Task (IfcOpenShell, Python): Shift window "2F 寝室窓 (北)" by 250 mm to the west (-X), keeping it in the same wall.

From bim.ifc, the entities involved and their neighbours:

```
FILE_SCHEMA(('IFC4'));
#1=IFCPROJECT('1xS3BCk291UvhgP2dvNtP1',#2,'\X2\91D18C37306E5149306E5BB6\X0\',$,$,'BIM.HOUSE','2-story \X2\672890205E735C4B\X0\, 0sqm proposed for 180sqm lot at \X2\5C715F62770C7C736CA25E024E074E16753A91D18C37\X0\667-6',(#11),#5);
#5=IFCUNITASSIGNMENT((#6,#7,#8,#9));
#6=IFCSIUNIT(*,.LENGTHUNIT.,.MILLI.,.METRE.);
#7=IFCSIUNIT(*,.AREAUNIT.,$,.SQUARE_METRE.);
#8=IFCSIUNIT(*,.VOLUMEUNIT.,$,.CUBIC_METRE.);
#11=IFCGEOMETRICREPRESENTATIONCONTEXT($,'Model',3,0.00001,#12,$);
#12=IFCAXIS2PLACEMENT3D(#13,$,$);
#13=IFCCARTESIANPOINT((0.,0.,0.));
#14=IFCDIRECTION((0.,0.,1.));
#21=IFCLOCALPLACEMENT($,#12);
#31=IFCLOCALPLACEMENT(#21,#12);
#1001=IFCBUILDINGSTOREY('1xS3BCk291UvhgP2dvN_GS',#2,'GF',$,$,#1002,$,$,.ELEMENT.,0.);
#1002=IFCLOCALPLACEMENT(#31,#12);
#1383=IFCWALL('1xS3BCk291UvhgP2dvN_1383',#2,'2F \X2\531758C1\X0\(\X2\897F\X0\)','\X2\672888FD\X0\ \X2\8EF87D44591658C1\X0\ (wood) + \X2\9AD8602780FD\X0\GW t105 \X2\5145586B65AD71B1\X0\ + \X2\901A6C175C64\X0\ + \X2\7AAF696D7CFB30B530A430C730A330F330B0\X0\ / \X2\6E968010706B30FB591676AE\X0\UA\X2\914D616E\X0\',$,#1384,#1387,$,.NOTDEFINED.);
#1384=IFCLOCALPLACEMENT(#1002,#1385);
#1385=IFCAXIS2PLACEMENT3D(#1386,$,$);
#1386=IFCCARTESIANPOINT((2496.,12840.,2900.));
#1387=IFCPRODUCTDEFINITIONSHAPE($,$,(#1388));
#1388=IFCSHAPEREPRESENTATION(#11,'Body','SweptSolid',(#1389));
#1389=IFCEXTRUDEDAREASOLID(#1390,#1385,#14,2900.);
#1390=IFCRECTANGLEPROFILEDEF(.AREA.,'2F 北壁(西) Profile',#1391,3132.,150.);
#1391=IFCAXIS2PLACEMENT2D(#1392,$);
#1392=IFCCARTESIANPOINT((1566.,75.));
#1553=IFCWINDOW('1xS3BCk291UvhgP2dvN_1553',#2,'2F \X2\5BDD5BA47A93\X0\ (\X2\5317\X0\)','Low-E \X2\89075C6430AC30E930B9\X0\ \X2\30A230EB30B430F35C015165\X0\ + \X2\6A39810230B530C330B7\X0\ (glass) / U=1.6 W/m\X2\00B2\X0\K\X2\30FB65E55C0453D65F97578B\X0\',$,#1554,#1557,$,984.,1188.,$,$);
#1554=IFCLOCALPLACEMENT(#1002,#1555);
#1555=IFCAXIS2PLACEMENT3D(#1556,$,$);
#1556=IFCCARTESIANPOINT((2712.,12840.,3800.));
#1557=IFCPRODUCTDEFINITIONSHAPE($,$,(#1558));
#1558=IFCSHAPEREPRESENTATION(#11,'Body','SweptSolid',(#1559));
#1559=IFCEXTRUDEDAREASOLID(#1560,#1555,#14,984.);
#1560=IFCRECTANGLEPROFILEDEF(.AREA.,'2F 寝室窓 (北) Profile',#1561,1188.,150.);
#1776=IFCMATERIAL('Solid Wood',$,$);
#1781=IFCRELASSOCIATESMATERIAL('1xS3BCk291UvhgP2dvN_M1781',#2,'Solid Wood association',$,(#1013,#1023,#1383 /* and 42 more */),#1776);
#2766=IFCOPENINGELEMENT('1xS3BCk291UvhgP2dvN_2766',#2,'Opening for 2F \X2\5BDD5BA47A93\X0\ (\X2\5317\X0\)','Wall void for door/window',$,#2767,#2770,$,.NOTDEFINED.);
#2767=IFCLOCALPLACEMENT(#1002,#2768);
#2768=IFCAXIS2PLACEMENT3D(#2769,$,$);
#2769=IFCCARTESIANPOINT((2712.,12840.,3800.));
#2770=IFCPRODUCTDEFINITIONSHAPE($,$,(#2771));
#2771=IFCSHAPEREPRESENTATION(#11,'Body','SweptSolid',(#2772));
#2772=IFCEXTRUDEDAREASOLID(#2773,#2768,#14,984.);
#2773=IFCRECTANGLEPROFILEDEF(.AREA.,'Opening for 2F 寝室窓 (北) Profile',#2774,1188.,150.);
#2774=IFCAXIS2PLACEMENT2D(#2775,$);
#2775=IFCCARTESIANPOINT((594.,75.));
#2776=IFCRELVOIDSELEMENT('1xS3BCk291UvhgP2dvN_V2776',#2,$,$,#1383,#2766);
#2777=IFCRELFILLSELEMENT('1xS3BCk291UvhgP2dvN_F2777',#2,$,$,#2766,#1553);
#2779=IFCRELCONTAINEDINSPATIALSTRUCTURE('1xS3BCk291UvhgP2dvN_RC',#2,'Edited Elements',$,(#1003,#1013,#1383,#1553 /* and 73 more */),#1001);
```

```python
import ifcopenshell
import ifcopenshell.api.geometry
import ifcopenshell.util.placement
import ifcopenshell.util.unit

model = ifcopenshell.open("bim.ifc")
unit_scale = ifcopenshell.util.unit.calculate_unit_scale(model)

window = model.by_id(1553)
opening = window.FillsVoids[0].RelatingOpeningElement
wall = opening.VoidsElements[0].RelatingBuildingElement

wall_matrix = ifcopenshell.util.placement.get_local_placement(wall.ObjectPlacement)
shift = wall_matrix[:3, 0] * -0.25 / unit_scale
before = ifcopenshell.util.placement.get_local_placement(window.ObjectPlacement)[:3, 3].copy()

# The window is not placed relative to its opening, so move both.
for product in (opening, window):
    matrix = ifcopenshell.util.placement.get_local_placement(product.ObjectPlacement)
    matrix[:3, 3] += shift
    ifcopenshell.api.geometry.edit_object_placement(model, product=product, matrix=matrix, is_si=False)

after = ifcopenshell.util.placement.get_local_placement(window.ObjectPlacement)[:3, 3]
print("window moved by", (after - before).round(3) + 0.0)

model.write("bim_v2.ifc")
```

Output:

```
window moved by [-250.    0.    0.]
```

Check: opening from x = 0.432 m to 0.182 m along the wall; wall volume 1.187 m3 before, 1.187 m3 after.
